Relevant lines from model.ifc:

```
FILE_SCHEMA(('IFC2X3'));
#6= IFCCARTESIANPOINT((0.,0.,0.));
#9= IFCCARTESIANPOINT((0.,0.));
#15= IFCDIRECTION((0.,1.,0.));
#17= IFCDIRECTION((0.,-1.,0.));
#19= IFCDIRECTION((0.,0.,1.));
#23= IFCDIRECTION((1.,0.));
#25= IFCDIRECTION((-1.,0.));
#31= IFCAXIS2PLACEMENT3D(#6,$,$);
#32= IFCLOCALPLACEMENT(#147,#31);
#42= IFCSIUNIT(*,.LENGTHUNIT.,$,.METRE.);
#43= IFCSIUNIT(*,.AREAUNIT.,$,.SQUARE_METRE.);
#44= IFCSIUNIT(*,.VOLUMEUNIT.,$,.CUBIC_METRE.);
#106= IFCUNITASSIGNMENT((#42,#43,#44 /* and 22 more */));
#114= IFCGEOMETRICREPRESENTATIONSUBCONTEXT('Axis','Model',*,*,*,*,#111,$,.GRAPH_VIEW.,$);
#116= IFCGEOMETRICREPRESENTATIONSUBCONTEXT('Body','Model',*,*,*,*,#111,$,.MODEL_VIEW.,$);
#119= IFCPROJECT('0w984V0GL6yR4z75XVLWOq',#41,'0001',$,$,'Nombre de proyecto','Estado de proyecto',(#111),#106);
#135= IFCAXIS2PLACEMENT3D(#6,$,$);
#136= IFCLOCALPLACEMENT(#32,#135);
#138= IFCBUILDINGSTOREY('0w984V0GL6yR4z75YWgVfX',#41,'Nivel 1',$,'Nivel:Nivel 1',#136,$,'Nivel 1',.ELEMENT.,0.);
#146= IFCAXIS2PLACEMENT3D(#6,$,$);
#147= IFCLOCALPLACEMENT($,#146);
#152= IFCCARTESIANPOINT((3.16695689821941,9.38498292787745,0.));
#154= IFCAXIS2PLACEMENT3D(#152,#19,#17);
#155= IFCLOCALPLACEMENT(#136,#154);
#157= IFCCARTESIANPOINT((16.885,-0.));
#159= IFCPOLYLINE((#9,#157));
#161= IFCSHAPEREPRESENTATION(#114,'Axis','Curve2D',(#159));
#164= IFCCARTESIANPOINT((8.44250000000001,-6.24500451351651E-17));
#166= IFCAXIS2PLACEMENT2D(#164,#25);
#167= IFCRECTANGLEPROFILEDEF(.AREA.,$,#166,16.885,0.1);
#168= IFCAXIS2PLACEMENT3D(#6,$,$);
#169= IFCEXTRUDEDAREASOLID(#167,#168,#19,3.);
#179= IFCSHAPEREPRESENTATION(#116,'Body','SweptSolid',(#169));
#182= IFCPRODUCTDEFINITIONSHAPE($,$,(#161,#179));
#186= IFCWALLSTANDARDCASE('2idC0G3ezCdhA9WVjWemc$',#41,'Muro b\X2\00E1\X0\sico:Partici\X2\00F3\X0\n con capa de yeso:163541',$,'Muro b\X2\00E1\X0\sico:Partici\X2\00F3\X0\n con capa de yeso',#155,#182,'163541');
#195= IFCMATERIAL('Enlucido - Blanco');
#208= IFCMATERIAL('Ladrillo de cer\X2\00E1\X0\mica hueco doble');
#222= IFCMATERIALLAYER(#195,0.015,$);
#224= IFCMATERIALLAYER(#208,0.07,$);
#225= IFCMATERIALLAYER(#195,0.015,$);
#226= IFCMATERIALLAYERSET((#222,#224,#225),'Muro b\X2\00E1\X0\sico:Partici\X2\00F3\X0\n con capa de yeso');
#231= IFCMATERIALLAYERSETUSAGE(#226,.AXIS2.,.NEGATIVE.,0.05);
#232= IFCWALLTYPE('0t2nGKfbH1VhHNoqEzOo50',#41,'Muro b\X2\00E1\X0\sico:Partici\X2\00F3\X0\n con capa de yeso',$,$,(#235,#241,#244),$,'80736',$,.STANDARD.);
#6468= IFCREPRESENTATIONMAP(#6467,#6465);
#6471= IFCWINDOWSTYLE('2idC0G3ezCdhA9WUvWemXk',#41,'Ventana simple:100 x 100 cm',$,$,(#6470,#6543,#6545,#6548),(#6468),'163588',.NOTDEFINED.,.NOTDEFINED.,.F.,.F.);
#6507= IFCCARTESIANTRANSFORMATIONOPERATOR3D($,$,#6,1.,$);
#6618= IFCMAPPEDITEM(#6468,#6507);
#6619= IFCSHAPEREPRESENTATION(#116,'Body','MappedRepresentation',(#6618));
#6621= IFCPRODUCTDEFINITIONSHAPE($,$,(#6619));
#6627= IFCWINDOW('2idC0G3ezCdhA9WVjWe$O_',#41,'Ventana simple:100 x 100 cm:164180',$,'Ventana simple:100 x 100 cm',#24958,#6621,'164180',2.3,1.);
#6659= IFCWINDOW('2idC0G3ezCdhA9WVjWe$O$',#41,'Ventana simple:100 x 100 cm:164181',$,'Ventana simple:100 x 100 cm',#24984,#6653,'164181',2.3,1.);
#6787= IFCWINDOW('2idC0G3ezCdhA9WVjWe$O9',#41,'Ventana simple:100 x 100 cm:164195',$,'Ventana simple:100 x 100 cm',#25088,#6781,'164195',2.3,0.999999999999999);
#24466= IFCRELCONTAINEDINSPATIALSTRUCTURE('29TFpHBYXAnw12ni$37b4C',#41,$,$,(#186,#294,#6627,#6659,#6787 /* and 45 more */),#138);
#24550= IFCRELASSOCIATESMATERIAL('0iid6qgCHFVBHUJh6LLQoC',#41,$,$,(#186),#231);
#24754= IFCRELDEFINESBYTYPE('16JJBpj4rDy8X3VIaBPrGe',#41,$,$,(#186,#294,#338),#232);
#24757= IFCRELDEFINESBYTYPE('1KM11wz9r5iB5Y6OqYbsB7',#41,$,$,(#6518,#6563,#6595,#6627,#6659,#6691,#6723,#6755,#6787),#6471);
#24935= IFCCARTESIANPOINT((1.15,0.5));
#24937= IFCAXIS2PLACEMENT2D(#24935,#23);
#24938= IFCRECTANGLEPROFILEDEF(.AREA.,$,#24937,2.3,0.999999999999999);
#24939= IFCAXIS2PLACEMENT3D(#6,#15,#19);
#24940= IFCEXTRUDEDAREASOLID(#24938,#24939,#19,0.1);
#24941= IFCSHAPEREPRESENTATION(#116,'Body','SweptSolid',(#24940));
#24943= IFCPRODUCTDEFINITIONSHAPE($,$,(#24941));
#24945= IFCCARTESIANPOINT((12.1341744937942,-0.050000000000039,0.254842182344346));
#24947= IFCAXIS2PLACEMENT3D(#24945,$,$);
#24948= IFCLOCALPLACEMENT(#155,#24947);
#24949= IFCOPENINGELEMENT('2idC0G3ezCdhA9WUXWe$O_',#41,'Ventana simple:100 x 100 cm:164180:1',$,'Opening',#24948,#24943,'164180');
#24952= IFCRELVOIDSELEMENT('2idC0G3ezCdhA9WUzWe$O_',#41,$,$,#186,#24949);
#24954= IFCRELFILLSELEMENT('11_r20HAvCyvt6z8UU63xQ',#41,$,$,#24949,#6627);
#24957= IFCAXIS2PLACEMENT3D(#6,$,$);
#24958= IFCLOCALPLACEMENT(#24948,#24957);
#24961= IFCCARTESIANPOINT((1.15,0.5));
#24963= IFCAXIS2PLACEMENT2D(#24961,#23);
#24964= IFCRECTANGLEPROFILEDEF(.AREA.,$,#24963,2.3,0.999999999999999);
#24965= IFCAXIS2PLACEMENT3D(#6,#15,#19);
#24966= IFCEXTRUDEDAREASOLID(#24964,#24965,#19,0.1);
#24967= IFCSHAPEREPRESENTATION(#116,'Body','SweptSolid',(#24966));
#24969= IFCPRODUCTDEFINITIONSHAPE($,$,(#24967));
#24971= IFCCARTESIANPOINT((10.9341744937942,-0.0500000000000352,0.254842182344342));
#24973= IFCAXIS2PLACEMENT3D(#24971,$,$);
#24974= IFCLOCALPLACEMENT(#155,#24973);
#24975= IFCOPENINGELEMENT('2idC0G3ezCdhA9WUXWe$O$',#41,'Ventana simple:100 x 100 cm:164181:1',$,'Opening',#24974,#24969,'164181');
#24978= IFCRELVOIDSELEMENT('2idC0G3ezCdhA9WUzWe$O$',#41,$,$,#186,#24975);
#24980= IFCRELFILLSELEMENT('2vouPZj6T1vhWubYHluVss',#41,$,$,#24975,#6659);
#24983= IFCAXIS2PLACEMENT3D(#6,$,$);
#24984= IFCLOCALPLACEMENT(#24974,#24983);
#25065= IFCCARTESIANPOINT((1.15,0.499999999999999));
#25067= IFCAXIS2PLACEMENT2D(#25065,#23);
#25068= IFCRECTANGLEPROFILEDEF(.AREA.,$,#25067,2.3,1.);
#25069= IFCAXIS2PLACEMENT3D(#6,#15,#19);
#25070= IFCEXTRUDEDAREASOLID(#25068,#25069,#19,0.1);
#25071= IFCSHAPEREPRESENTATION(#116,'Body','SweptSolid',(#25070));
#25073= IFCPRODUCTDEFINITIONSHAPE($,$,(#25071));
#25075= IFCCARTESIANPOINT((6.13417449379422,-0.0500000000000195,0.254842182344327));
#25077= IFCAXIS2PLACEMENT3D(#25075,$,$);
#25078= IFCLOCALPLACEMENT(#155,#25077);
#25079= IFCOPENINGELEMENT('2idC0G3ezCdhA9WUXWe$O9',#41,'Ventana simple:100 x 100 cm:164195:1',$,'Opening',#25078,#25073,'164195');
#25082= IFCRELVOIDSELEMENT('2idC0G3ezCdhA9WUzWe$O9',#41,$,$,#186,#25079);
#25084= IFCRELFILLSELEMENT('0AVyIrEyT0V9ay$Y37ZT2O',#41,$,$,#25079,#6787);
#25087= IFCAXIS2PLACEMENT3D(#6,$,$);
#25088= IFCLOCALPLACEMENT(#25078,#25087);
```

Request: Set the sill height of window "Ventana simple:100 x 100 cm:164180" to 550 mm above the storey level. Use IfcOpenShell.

```python
import numpy as np
import ifcopenshell
import ifcopenshell.api.geometry
import ifcopenshell.geom
import ifcopenshell.util.element
import ifcopenshell.util.placement
import ifcopenshell.util.shape
import ifcopenshell.util.unit

model = ifcopenshell.open("model.ifc")
unit_scale = ifcopenshell.util.unit.calculate_unit_scale(model)

window = model.by_guid("2idC0G3ezCdhA9WVjWe$O_")
opening = window.FillsVoids[0].RelatingOpeningElement
storey = ifcopenshell.util.element.get_container(window, ifc_class="IfcBuildingStorey")
level = ifcopenshell.util.placement.get_local_placement(storey.ObjectPlacement)[2, 3]

# The opening's origin need not be at the sill, so measure its lowest point.
shape = ifcopenshell.geom.create_shape(ifcopenshell.geom.settings(), opening)
bottom = ifcopenshell.util.shape.get_shape_bottom_elevation(shape, shape.geometry) / unit_scale
dz = level + 0.55 / unit_scale - bottom

shift = np.array([0.0, 0.0, dz])
# The window is placed relative to its opening, so it follows when the opening moves.
matrix = ifcopenshell.util.placement.get_local_placement(opening.ObjectPlacement)
matrix[:3, 3] += shift
ifcopenshell.api.geometry.edit_object_placement(
    model, product=opening, matrix=matrix, is_si=False, should_transform_children=True
)

print(f"moved by {dz * unit_scale:+.3f} m")

model.write("model_v2.ifc")
```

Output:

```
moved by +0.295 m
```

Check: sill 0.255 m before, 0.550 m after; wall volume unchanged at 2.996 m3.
